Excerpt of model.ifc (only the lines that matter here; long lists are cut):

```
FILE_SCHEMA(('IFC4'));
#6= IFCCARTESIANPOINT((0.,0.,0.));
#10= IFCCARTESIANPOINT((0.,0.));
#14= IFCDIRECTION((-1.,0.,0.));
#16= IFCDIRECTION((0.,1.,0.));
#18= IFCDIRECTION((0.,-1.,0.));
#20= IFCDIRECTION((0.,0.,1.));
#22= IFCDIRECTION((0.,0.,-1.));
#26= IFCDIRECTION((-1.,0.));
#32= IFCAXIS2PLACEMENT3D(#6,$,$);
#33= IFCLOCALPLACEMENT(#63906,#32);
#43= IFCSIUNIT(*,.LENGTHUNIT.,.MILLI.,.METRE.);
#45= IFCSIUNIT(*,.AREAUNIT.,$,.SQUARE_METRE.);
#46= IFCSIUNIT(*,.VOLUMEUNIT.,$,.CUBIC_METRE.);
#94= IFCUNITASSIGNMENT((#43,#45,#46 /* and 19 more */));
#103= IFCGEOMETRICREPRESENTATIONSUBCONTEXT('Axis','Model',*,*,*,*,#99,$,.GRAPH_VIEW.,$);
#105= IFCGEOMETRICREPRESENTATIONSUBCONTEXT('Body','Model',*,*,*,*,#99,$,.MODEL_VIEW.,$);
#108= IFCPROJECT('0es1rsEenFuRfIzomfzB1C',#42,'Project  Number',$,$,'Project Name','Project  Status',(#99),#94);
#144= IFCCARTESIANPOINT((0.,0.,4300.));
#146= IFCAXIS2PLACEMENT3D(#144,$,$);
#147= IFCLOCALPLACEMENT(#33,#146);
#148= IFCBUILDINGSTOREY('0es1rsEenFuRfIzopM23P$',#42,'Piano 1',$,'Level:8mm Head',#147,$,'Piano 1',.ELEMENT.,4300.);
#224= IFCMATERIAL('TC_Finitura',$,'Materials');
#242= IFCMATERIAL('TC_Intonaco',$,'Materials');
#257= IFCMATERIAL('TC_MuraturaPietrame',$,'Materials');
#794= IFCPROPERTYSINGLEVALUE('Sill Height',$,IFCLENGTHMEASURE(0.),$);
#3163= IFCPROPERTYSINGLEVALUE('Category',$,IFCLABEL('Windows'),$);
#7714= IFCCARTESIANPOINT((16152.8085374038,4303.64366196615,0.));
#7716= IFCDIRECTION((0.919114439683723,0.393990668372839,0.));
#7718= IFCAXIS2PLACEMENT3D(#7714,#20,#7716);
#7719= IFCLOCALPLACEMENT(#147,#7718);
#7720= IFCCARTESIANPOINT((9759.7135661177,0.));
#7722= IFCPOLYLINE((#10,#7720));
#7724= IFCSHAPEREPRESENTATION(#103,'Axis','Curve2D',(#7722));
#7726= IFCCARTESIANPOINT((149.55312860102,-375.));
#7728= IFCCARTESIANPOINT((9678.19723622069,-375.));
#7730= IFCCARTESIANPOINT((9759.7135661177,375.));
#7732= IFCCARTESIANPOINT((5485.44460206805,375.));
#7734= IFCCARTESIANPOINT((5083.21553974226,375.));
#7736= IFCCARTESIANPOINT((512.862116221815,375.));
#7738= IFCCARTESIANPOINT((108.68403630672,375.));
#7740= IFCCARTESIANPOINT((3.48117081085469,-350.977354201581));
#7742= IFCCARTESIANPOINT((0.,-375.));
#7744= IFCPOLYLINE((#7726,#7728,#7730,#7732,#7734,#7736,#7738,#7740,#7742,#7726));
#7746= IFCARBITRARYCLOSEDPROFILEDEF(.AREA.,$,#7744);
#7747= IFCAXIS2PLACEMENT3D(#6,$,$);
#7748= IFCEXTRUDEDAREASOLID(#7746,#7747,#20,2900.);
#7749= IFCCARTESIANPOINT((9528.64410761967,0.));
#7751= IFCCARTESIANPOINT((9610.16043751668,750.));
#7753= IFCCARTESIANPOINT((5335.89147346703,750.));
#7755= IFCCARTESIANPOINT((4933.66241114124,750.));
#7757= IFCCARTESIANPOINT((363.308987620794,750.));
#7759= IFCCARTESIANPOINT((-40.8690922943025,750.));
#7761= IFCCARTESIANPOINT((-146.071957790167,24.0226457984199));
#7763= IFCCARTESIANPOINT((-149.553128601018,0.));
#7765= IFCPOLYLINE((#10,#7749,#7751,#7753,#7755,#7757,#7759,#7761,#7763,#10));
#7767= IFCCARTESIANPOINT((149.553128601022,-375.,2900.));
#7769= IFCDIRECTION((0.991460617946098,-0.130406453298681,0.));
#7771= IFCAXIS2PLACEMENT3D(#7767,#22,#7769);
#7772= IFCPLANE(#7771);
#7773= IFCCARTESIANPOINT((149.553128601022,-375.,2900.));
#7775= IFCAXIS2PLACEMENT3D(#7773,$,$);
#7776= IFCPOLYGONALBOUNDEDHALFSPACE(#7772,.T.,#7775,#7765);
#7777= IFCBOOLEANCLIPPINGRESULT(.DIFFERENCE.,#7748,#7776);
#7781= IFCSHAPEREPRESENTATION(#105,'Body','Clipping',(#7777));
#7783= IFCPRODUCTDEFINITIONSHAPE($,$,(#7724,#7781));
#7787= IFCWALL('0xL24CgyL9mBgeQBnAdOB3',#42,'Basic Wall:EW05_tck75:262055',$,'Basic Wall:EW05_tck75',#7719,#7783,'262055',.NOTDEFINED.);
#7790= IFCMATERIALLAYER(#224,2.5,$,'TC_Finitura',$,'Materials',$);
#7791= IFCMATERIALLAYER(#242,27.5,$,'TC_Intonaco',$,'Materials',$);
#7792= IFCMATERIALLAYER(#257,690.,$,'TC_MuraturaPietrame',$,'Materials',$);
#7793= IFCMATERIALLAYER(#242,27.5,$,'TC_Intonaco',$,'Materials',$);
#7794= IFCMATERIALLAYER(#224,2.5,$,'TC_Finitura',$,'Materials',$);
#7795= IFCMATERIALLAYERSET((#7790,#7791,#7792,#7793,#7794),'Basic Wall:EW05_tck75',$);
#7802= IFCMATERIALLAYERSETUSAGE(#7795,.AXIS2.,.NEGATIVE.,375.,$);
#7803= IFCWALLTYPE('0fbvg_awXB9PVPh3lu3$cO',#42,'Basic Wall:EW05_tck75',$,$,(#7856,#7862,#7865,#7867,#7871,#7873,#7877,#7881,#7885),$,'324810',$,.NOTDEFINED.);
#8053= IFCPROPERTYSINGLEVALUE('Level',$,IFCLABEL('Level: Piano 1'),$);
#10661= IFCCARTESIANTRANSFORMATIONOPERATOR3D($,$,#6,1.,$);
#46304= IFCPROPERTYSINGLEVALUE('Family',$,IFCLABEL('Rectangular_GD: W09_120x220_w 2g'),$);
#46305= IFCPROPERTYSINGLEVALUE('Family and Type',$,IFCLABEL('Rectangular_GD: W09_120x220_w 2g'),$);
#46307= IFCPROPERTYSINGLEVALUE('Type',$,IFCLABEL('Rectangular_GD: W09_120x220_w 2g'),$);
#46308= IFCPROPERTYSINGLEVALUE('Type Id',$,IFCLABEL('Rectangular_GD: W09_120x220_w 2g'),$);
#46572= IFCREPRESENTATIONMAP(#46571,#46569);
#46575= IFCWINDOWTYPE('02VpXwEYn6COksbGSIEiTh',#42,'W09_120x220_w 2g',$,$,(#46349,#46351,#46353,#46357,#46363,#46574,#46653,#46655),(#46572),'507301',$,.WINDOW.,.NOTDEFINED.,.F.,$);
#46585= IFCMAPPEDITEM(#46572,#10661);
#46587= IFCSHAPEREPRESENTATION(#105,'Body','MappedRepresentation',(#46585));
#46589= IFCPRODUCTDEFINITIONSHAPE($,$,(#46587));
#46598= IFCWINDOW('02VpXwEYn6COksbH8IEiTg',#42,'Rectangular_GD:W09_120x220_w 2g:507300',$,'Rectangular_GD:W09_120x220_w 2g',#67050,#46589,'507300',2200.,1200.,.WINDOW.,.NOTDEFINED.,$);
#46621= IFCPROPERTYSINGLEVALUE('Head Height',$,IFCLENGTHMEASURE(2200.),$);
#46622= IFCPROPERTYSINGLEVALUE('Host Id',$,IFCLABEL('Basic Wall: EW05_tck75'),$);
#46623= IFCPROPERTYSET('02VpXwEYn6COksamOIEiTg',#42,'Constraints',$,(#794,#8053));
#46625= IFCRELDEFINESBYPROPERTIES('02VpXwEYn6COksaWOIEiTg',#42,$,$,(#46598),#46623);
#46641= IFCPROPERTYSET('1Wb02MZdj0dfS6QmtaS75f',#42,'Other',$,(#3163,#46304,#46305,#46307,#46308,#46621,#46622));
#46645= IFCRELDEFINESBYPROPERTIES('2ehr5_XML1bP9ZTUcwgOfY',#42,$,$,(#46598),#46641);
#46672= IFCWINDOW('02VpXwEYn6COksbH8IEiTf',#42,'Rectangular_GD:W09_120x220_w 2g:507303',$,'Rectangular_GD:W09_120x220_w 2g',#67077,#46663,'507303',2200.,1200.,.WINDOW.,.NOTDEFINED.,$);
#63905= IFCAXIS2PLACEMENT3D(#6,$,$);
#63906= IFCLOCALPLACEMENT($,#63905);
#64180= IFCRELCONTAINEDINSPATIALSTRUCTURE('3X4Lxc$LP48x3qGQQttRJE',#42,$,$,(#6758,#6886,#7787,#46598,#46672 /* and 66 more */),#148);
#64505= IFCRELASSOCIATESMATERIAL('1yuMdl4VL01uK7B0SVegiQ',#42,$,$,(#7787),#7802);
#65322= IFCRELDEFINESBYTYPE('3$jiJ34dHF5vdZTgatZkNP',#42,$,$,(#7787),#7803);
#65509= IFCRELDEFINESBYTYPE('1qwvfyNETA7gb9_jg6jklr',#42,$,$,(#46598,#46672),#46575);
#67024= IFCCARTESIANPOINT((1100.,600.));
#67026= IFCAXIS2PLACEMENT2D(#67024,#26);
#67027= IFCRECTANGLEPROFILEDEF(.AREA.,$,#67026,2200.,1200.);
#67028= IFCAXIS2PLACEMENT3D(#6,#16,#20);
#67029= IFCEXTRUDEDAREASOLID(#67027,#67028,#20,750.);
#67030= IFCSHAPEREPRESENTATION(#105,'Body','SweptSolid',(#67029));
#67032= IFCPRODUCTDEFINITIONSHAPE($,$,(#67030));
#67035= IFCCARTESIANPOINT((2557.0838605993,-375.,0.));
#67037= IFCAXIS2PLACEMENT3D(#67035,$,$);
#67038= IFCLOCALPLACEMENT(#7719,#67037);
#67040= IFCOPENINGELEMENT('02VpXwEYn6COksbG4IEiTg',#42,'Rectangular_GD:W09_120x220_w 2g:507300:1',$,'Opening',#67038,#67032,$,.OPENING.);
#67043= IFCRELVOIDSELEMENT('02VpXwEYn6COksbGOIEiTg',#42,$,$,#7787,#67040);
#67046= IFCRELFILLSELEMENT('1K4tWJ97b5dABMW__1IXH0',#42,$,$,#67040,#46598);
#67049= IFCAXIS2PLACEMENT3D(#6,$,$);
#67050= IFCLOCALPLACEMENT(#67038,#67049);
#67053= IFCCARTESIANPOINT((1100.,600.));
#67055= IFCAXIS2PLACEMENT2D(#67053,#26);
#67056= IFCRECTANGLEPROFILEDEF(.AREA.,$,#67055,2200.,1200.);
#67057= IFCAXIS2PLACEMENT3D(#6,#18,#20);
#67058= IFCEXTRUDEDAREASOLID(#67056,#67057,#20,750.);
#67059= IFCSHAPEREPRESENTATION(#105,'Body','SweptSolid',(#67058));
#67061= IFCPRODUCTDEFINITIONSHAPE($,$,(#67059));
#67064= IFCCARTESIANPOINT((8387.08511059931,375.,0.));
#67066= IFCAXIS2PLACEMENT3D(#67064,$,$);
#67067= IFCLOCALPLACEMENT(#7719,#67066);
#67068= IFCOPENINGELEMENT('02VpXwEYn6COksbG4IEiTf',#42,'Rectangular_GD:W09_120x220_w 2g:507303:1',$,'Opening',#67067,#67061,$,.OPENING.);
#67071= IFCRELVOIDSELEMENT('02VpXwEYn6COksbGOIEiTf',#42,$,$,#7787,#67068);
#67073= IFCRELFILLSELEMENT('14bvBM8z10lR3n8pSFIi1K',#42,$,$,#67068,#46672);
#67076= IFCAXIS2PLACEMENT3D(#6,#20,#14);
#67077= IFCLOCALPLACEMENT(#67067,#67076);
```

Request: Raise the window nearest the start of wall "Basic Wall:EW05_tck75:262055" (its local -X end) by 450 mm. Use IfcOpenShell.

```python
import numpy as np
import ifcopenshell
import ifcopenshell.api.geometry
import ifcopenshell.api.pset
import ifcopenshell.util.element
import ifcopenshell.util.placement
import ifcopenshell.util.unit

model = ifcopenshell.open("model.ifc")
unit_scale = ifcopenshell.util.unit.calculate_unit_scale(model)

window = model.by_guid("02VpXwEYn6COksbH8IEiTg")
opening = window.FillsVoids[0].RelatingOpeningElement
dz = 450.0

shift = np.array([0.0, 0.0, dz])
# The window is placed relative to its opening, so it follows when the opening moves.
matrix = ifcopenshell.util.placement.get_local_placement(opening.ObjectPlacement)
matrix[:3, 3] += shift
ifcopenshell.api.geometry.edit_object_placement(
    model, product=opening, matrix=matrix, is_si=False, should_transform_children=True
)

# Keep the stored heights in step.
pset = model.by_id(ifcopenshell.util.element.get_pset(window, "Constraints", should_inherit=False)["id"])
ifcopenshell.api.pset.edit_pset(model, pset=pset, properties={
    "Sill Height": model.create_entity("IfcLengthMeasure", ifcopenshell.util.element.get_pset(window, "Constraints", "Sill Height") + dz),
})
pset = model.by_id(ifcopenshell.util.element.get_pset(window, "Other", should_inherit=False)["id"])
ifcopenshell.api.pset.edit_pset(model, pset=pset, properties={
    "Head Height": model.create_entity("IfcLengthMeasure", ifcopenshell.util.element.get_pset(window, "Other", "Head Height") + dz),
})

print(f"moved by {dz * unit_scale:+.3f} m")

model.write("model_edited.ifc")
```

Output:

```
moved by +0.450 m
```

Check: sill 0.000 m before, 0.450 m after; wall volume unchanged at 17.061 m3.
